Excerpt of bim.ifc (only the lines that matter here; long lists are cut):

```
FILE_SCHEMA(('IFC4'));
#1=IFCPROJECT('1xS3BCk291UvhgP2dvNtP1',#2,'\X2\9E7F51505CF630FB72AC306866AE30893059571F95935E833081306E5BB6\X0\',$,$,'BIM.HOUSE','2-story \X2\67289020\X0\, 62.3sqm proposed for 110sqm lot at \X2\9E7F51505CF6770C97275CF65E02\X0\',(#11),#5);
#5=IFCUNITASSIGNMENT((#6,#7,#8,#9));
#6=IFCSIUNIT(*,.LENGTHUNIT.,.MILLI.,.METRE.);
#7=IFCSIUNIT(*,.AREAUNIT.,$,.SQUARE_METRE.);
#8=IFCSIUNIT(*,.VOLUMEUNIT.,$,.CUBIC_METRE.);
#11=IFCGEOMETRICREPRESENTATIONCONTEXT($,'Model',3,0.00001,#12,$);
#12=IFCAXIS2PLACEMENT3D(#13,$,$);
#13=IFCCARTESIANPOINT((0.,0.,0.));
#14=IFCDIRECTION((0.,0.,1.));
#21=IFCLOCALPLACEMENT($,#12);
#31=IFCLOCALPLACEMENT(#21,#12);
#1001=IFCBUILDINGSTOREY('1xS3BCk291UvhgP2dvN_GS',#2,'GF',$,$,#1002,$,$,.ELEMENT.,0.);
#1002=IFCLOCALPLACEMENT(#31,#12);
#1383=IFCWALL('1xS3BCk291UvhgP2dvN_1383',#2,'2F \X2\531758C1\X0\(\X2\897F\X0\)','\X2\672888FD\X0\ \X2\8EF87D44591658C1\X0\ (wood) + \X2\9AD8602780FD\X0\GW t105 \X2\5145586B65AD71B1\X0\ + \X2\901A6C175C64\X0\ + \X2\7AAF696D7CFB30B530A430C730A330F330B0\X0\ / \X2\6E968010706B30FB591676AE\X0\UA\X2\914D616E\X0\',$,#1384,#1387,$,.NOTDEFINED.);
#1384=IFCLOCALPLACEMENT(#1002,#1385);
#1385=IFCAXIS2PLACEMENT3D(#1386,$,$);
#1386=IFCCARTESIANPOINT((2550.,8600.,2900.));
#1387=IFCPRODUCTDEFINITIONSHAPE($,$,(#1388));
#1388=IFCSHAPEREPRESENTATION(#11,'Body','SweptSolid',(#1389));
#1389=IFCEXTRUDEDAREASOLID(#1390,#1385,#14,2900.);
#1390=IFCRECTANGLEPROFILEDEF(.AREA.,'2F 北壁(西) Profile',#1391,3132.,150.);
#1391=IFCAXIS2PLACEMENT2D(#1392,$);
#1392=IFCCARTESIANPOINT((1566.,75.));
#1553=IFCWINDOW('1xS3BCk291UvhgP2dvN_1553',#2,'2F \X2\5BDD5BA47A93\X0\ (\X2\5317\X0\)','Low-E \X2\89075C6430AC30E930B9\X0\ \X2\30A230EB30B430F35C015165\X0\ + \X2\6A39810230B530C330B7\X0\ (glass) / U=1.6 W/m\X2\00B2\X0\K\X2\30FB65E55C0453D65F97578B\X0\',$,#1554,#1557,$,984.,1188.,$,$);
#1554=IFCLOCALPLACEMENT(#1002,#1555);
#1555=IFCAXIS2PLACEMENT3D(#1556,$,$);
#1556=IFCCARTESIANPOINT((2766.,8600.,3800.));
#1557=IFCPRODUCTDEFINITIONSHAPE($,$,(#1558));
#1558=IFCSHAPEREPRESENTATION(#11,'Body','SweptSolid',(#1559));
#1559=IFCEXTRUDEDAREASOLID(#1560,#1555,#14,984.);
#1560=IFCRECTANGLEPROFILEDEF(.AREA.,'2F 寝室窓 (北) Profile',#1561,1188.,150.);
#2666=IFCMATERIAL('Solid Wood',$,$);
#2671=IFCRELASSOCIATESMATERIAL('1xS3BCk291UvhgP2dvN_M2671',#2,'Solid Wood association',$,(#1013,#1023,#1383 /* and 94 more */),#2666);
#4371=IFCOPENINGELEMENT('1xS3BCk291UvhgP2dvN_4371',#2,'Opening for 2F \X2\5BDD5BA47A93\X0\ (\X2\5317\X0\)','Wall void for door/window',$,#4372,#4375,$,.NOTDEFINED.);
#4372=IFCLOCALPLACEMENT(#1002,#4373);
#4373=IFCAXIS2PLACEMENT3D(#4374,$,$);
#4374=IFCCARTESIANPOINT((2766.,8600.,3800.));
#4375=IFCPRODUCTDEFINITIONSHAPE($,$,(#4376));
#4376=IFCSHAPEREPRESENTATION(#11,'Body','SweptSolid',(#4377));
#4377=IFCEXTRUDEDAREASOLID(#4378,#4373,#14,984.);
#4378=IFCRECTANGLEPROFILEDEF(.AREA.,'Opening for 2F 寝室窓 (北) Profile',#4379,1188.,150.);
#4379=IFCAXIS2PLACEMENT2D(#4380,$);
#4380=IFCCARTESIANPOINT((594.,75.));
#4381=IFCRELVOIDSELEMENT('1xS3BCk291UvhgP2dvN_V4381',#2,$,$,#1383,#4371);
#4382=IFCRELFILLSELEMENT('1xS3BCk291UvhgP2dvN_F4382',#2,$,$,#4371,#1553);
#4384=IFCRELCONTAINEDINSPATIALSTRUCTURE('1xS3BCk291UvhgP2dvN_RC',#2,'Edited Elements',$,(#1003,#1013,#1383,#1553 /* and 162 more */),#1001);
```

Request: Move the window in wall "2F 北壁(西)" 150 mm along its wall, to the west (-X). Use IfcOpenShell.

```python
import ifcopenshell
import ifcopenshell.api.geometry
import ifcopenshell.util.placement

model = ifcopenshell.open("bim.ifc")

window = model.by_guid("1xS3BCk291UvhgP2dvN_1553")
opening = window.FillsVoids[0].RelatingOpeningElement
wall = opening.VoidsElements[0].RelatingBuildingElement

wall_matrix = ifcopenshell.util.placement.get_local_placement(wall.ObjectPlacement)
shift = wall_matrix[:3, 0] * -150.0
before = ifcopenshell.util.placement.get_local_placement(window.ObjectPlacement)[:3, 3].copy()

# The window is not placed relative to its opening, so move both.
for product in (opening, window):
    matrix = ifcopenshell.util.placement.get_local_placement(product.ObjectPlacement)
    matrix[:3, 3] += shift
    ifcopenshell.api.geometry.edit_object_placement(model, product=product, matrix=matrix, is_si=False)

after = ifcopenshell.util.placement.get_local_placement(window.ObjectPlacement)[:3, 3]
print("window moved by", (after - before).round(3) + 0.0)

model.write("bim_rev.ifc")
```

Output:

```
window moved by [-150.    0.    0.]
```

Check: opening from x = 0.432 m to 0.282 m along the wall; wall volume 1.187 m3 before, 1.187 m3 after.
